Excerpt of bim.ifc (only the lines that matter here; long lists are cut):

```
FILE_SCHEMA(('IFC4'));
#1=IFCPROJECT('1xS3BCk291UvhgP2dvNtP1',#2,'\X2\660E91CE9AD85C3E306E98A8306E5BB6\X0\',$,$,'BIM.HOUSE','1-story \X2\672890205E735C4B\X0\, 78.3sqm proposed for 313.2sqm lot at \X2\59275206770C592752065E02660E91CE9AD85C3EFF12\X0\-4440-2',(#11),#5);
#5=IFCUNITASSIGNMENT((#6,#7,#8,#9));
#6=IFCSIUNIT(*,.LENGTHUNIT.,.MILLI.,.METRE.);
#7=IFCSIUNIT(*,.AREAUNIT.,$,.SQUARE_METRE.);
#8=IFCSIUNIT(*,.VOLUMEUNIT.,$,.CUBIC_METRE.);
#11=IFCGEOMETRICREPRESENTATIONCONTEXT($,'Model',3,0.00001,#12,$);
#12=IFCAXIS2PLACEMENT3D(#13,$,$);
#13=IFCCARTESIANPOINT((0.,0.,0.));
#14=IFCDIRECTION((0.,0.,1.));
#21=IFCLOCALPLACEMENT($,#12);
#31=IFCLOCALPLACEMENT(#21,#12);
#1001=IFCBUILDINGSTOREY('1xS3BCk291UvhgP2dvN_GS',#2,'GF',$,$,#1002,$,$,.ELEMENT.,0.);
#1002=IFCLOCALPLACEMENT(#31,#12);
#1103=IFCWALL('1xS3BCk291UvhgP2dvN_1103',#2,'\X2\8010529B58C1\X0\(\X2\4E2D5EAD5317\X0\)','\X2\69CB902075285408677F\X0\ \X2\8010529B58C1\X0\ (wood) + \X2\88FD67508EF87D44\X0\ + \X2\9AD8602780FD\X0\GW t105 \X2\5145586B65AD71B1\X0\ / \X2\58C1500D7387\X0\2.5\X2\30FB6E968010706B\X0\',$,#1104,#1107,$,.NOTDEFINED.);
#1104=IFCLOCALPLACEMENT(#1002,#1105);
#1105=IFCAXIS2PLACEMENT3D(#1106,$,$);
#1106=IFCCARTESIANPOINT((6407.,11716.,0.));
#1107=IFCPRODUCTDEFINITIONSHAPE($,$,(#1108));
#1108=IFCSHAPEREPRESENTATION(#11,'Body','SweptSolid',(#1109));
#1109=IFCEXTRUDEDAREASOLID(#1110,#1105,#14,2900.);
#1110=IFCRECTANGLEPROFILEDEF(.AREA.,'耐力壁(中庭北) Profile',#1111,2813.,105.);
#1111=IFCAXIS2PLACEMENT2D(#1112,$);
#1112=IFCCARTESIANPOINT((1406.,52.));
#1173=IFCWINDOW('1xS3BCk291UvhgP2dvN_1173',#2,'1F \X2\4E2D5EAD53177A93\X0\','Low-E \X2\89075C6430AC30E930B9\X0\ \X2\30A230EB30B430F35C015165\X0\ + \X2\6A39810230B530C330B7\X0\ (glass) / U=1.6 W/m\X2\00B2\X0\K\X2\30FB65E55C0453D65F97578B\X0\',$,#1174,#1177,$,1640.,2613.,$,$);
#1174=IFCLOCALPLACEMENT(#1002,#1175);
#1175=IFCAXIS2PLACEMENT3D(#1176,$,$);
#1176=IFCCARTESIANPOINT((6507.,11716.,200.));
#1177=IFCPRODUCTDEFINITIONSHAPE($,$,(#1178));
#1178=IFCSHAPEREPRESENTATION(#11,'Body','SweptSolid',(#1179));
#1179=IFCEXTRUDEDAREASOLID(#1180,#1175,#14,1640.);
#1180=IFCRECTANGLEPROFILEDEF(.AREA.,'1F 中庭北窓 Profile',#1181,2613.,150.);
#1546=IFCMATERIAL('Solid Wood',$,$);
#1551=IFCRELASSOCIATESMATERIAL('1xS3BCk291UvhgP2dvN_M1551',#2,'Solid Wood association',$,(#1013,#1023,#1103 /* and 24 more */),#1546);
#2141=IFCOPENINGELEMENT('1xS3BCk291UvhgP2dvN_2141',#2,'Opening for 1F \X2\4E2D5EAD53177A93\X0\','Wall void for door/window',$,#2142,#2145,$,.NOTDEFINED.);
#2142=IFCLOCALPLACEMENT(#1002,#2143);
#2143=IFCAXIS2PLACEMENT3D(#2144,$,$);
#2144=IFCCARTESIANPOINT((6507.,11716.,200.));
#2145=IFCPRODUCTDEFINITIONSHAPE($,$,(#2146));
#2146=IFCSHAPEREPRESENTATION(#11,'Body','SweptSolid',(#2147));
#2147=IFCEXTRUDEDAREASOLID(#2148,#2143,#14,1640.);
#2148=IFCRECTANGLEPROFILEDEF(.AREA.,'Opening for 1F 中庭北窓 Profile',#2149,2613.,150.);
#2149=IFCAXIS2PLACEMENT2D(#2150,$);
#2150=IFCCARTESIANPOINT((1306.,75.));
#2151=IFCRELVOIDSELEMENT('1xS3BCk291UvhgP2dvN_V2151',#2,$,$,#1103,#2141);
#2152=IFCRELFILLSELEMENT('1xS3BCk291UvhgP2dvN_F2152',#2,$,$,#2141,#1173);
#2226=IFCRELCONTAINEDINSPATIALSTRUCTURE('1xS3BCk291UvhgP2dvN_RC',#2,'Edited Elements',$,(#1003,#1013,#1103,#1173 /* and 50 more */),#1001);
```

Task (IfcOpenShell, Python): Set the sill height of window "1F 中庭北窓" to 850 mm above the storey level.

```python
import numpy as np
import ifcopenshell
import ifcopenshell.api.geometry
import ifcopenshell.geom
import ifcopenshell.util.element
import ifcopenshell.util.placement
import ifcopenshell.util.shape
import ifcopenshell.util.unit

model = ifcopenshell.open("bim.ifc")
unit_scale = ifcopenshell.util.unit.calculate_unit_scale(model)

window = model.by_guid("1xS3BCk291UvhgP2dvN_1173")
opening = window.FillsVoids[0].RelatingOpeningElement
storey = ifcopenshell.util.element.get_container(window, ifc_class="IfcBuildingStorey")
level = ifcopenshell.util.placement.get_local_placement(storey.ObjectPlacement)[2, 3]

# The opening's origin need not be at the sill, so measure its lowest point.
shape = ifcopenshell.geom.create_shape(ifcopenshell.geom.settings(), opening)
bottom = ifcopenshell.util.shape.get_shape_bottom_elevation(shape, shape.geometry) / unit_scale
dz = level + 850.0 - bottom

shift = np.array([0.0, 0.0, dz])
# The window is not placed relative to its opening, so move both.
for product in (opening, window):
    matrix = ifcopenshell.util.placement.get_local_placement(product.ObjectPlacement)
    matrix[:3, 3] += shift
    ifcopenshell.api.geometry.edit_object_placement(model, product=product, matrix=matrix, is_si=False)

print(f"moved by {dz * unit_scale:+.3f} m")

model.write("bim-out.ifc")
```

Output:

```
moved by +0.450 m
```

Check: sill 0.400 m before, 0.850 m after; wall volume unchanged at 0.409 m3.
